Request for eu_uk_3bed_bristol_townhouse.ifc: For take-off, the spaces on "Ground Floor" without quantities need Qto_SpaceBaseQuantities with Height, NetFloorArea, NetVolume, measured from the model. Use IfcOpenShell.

First a look at what the model holds.

```python
import ifcopenshell
import ifcopenshell.util.element
import ifcopenshell.util.unit

model = ifcopenshell.open("eu_uk_3bed_bristol_townhouse.ifc")
print(model.schema)
for unit_type in ("LENGTHUNIT", "AREAUNIT", "VOLUMEUNIT"):
    print(unit_type, ifcopenshell.util.unit.calculate_unit_scale(model, unit_type))
storey = next(s for s in model.by_type("IfcBuildingStorey") if s.Name == "Ground Floor")
spaces = [e for e in ifcopenshell.util.element.get_decomposition(storey) if e.is_a("IfcSpace")]
for e in sorted(spaces, key=lambda e: e.id()):
    print(e.id(), e.is_a(), e.Name, list(ifcopenshell.util.element.get_psets(e, qtos_only=True)), sep=" | ")
```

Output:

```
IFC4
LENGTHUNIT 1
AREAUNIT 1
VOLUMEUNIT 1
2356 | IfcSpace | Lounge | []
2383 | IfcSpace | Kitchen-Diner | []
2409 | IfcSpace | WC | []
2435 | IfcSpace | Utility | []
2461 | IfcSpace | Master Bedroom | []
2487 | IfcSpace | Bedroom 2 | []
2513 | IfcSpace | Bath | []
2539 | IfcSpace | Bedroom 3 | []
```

```python
import ifcopenshell
import ifcopenshell.api.pset
import ifcopenshell.geom
import ifcopenshell.util.element
import ifcopenshell.util.shape
import ifcopenshell.util.unit

model = ifcopenshell.open("eu_uk_3bed_bristol_townhouse.ifc")
unit_scale = ifcopenshell.util.unit.calculate_unit_scale(model)
area_scale = ifcopenshell.util.unit.calculate_unit_scale(model, "AREAUNIT")
volume_scale = ifcopenshell.util.unit.calculate_unit_scale(model, "VOLUMEUNIT")
settings = ifcopenshell.geom.settings()

storey = next(s for s in model.by_type("IfcBuildingStorey") if s.Name == "Ground Floor")
spaces = [e for e in ifcopenshell.util.element.get_decomposition(storey) if e.is_a("IfcSpace")]

for e in sorted(spaces, key=lambda e: e.id()):
    if ifcopenshell.util.element.get_psets(e, qtos_only=True, should_inherit=False):
        continue
    # Geometry comes back in metres, in the element's own axes.
    shape = ifcopenshell.geom.create_shape(settings, e)
    values = {
        "Height": ifcopenshell.util.shape.get_z(shape.geometry) / unit_scale,
        "NetFloorArea": ifcopenshell.util.shape.get_footprint_area(shape.geometry) / area_scale,
        "NetVolume": ifcopenshell.util.shape.get_volume(shape.geometry) / volume_scale,
    }
    qto = ifcopenshell.api.pset.add_qto(model, product=e, name="Qto_SpaceBaseQuantities")
    ifcopenshell.api.pset.edit_qto(model, qto=qto, properties=values)
    print(e.id(), {k: round(v, 3) for k, v in values.items()})

model.write("eu_uk_3bed_bristol_townhouse-out.ifc")
```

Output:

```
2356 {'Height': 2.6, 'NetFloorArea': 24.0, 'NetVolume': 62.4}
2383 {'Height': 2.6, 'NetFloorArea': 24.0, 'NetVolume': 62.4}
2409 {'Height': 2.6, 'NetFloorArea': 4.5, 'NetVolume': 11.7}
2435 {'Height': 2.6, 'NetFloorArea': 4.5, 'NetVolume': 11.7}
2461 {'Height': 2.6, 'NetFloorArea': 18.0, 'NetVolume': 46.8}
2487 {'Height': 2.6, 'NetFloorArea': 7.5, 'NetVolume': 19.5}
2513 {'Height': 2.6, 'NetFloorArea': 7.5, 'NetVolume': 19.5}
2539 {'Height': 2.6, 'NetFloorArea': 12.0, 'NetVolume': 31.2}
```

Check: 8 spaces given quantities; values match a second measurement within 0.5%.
